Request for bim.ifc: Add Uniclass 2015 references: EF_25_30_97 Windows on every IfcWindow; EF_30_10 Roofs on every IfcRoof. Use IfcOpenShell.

First a look at what the model holds.

```python
import ifcopenshell

model = ifcopenshell.open("bim.ifc")
print(model.schema)
print("classifications:", [c.Name for c in model.by_type("IfcClassification")])
for ifc_class in ("IfcDoor", "IfcRoof", "IfcStair", "IfcWall", "IfcWindow"):
    print(ifc_class, len(model.by_type(ifc_class)))
```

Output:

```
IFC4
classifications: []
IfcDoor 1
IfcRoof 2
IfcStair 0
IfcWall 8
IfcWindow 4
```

```python
import ifcopenshell
import ifcopenshell.api.classification

model = ifcopenshell.open("bim.ifc")

system = ifcopenshell.api.classification.add_classification(model, classification="Uniclass 2015")

codes = {
    "IfcWindow": ("EF_25_30_97", "Windows"),
    "IfcRoof": ("EF_30_10", "Roofs"),
}
for ifc_class, (code, name) in codes.items():
    products = model.by_type(ifc_class)
    ifcopenshell.api.classification.add_reference(
        model, products=products, classification=system, identification=code, name=name
    )
    print(code, len(products))

model.write("bim_v2.ifc")
```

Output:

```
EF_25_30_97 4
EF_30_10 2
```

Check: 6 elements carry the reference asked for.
